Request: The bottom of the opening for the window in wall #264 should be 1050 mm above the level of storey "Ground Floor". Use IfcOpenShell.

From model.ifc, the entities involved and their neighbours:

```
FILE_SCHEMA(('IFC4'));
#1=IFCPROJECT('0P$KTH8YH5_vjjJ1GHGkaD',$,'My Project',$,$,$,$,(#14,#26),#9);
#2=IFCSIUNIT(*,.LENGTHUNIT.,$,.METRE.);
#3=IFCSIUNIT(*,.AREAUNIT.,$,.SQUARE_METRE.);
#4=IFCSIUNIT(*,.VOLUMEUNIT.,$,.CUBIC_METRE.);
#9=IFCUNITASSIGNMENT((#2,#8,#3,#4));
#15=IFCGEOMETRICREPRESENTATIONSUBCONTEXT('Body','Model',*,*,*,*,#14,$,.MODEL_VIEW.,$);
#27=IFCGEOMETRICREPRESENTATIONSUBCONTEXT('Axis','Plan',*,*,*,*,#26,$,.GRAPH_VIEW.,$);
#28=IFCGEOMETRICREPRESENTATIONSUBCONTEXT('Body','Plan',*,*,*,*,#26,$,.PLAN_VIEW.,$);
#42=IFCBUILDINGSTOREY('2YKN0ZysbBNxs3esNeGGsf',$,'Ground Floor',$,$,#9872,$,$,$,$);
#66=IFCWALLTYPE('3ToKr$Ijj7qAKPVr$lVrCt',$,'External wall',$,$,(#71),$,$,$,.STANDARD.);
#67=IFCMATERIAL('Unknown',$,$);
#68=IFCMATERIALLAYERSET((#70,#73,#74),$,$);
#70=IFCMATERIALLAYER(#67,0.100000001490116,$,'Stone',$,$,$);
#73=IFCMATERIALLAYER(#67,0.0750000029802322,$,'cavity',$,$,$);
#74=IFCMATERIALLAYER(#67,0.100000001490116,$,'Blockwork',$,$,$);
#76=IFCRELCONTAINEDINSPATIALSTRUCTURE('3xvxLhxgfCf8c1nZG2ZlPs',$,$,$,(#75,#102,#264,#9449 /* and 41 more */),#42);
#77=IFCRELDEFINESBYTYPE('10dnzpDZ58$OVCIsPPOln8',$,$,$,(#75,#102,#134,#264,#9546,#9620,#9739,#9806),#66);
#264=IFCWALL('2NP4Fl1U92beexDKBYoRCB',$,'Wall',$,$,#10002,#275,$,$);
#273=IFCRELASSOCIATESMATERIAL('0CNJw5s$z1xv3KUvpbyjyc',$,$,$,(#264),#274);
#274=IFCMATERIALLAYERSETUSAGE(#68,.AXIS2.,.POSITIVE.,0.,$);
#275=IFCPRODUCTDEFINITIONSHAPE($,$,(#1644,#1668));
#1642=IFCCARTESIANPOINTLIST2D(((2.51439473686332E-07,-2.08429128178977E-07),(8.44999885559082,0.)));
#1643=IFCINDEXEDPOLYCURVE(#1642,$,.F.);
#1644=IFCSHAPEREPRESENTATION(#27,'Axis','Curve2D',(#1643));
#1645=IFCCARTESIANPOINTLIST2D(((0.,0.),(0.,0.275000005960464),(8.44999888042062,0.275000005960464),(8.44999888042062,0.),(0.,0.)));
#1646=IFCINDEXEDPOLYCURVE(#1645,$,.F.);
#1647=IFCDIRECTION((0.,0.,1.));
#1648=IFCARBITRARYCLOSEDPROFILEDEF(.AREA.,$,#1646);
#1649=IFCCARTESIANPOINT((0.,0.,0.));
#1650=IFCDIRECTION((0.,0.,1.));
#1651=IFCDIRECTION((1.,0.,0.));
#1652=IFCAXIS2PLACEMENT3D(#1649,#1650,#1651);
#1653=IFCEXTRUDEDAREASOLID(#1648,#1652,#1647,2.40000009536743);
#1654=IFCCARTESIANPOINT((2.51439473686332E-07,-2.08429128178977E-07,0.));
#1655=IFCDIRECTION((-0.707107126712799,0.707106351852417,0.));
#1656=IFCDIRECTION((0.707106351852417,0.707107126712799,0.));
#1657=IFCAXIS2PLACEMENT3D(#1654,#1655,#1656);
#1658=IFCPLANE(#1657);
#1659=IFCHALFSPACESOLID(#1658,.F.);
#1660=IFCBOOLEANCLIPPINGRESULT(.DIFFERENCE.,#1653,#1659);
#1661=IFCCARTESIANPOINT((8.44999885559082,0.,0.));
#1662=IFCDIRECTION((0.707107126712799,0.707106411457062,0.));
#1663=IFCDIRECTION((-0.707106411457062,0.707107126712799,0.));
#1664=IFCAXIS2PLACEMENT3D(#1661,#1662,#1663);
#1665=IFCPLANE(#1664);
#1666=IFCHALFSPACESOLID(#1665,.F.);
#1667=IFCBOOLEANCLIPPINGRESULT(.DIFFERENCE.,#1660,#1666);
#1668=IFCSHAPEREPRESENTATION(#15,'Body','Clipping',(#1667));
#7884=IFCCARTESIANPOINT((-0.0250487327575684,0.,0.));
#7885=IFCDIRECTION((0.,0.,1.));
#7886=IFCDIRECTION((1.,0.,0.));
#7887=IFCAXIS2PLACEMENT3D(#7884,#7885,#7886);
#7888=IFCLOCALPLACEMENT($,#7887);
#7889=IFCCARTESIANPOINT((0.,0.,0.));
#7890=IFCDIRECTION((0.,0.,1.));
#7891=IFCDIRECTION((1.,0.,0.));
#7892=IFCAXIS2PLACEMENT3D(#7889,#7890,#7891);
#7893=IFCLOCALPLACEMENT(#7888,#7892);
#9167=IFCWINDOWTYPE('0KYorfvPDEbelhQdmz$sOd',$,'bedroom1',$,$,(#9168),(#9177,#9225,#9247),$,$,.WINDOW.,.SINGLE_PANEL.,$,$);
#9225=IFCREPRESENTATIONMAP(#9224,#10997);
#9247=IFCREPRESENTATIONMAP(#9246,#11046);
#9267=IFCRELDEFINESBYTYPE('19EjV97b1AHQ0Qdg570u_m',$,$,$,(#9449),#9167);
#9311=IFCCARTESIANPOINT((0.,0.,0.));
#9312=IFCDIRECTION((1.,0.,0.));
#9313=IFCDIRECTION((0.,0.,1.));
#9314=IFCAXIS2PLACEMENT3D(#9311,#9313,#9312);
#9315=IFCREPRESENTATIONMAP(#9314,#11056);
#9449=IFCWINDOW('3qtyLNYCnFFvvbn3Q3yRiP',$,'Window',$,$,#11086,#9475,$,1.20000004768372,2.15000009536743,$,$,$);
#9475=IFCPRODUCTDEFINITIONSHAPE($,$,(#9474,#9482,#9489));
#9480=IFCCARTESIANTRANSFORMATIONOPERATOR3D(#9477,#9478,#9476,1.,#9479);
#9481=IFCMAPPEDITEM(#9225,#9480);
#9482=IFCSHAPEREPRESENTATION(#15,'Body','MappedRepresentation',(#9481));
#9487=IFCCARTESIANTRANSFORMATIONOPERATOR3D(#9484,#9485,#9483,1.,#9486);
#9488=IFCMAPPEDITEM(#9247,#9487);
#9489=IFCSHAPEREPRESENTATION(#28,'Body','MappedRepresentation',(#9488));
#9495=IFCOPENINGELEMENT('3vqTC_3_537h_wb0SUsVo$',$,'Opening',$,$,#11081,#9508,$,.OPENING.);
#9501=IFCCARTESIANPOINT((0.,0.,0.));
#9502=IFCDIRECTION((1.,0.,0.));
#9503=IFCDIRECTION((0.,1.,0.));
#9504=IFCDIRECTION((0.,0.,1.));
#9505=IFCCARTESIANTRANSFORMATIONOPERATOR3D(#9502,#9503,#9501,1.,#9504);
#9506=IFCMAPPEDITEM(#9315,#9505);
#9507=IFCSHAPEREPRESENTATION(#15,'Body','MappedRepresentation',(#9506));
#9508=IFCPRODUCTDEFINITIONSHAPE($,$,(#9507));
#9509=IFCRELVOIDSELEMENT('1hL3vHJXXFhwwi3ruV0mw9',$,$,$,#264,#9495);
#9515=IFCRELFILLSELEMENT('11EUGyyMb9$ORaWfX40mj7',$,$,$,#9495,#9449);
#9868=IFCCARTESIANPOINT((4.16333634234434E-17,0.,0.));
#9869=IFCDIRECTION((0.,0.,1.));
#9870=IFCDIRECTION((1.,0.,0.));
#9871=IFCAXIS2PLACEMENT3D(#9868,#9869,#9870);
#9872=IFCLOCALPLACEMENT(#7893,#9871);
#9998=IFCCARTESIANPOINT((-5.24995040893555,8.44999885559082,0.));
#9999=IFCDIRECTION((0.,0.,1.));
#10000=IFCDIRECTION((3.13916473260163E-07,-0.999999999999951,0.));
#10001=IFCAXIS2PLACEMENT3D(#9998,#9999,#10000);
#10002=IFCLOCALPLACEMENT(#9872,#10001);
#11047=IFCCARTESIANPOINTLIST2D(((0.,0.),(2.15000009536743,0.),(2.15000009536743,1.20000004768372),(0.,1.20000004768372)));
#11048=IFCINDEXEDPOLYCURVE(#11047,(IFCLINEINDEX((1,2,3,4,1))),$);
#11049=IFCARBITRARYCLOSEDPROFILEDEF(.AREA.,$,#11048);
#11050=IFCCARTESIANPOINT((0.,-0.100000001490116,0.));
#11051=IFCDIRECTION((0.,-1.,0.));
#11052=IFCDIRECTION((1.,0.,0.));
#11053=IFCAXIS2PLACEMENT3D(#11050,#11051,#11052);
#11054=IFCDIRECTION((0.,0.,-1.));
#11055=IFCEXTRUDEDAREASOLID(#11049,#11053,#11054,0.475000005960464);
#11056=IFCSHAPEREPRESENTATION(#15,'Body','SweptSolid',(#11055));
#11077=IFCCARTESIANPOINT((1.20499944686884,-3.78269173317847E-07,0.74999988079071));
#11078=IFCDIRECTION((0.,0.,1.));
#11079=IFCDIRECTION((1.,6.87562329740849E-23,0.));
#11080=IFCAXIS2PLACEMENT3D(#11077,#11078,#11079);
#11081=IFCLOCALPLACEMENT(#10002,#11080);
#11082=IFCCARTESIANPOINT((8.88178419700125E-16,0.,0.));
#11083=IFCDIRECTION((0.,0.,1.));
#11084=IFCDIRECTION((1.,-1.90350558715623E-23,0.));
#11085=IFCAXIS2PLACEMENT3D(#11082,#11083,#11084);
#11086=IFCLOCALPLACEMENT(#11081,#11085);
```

```python
import numpy as np
import ifcopenshell
import ifcopenshell.api.geometry
import ifcopenshell.geom
import ifcopenshell.util.element
import ifcopenshell.util.placement
import ifcopenshell.util.shape
import ifcopenshell.util.unit

model = ifcopenshell.open("model.ifc")
unit_scale = ifcopenshell.util.unit.calculate_unit_scale(model)

window = model.by_id(9449)
opening = window.FillsVoids[0].RelatingOpeningElement
storey = ifcopenshell.util.element.get_container(window, ifc_class="IfcBuildingStorey")
level = ifcopenshell.util.placement.get_local_placement(storey.ObjectPlacement)[2, 3]

# The opening's origin need not be at the sill, so measure its lowest point.
shape = ifcopenshell.geom.create_shape(ifcopenshell.geom.settings(), opening)
bottom = ifcopenshell.util.shape.get_shape_bottom_elevation(shape, shape.geometry) / unit_scale
dz = level + 1.05 / unit_scale - bottom

shift = np.array([0.0, 0.0, dz])
# The window is placed relative to its opening, so it follows when the opening moves.
matrix = ifcopenshell.util.placement.get_local_placement(opening.ObjectPlacement)
matrix[:3, 3] += shift
ifcopenshell.api.geometry.edit_object_placement(
    model, product=opening, matrix=matrix, is_si=False, should_transform_children=True
)

print(f"moved by {dz * unit_scale:+.3f} m")

model.write("model-out.ifc")
```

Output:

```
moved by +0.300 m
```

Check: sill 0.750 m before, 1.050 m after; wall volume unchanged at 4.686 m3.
